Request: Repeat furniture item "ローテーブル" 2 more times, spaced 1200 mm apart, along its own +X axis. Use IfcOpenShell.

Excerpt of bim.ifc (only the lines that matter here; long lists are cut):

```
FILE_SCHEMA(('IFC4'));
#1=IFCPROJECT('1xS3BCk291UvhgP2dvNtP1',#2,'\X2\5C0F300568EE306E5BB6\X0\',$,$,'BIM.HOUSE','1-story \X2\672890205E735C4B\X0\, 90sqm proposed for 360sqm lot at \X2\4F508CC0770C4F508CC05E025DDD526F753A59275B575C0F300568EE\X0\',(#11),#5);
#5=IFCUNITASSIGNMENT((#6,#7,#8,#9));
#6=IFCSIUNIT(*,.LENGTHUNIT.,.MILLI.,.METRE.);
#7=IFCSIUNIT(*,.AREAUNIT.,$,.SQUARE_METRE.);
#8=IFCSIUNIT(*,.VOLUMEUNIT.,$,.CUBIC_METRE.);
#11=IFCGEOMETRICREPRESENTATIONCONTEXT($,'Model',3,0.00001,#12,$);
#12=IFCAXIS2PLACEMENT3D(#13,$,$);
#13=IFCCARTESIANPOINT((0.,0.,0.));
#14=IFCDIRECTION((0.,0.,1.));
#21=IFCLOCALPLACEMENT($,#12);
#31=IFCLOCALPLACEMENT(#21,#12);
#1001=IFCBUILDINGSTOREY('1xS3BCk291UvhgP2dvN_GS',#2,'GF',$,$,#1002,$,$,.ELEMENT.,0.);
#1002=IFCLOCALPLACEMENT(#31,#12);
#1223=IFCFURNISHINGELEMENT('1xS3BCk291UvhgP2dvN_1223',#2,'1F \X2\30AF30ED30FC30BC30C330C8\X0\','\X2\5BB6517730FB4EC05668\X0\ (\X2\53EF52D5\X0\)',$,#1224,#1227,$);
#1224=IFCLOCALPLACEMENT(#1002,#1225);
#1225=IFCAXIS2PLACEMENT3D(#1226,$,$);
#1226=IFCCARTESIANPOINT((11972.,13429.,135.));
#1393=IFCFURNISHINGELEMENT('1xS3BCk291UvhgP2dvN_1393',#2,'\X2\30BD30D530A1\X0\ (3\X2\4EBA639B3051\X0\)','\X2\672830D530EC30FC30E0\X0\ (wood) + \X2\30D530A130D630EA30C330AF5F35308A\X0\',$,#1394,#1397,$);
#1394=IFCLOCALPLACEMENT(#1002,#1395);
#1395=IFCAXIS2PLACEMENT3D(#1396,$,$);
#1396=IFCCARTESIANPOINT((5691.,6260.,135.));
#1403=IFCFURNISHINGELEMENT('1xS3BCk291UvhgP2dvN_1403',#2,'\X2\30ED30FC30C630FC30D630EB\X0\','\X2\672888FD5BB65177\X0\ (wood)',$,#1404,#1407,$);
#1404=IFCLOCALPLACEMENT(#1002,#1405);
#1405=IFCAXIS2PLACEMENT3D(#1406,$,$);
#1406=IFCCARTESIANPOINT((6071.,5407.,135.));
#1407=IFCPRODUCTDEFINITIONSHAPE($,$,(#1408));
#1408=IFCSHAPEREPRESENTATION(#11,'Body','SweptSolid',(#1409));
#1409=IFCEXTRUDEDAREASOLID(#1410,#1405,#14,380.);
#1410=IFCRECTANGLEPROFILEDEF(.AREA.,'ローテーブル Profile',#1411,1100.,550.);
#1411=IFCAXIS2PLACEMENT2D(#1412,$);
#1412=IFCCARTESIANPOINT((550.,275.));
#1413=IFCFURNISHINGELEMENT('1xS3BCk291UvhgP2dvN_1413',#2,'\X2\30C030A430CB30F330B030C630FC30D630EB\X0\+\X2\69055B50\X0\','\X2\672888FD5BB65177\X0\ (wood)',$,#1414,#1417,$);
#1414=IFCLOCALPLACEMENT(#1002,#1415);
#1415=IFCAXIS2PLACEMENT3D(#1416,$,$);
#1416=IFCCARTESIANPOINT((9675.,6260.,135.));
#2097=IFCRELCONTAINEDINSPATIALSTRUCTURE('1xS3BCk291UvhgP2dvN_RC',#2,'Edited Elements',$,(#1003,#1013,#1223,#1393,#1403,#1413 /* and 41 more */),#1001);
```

```python
import ifcopenshell
import ifcopenshell.api.geometry
import ifcopenshell.api.root
import ifcopenshell.util.element
import ifcopenshell.util.placement
import ifcopenshell.util.unit

model = ifcopenshell.open("bim.ifc")
unit_scale = ifcopenshell.util.unit.calculate_unit_scale(model)


def reuse_history(source, copy):
    """copy_class also copies each property set's owner history, people and application; keep the originals."""
    for rel in copy.IsDefinedBy:
        if rel.is_a("IfcRelDefinesByProperties") and (history := rel.RelatingPropertyDefinition.OwnerHistory):
            rel.RelatingPropertyDefinition.OwnerHistory = source.OwnerHistory
            ifcopenshell.util.element.remove_deep2(model, history)


source = model.by_id(1403)
base = ifcopenshell.util.placement.get_local_placement(source.ObjectPlacement)
step = base[:3, 0] * 1.2 / unit_scale

for i in range(1, 3):
    copy = ifcopenshell.api.root.copy_class(model, product=source)
    copy.Representation = ifcopenshell.util.element.copy_deep(
        model, source.Representation, exclude=["IfcGeometricRepresentationContext", "IfcRepresentationMap"]
    )
    reuse_history(source, copy)
    matrix = base.copy()
    matrix[:3, 3] += i * step
    print("added at", matrix[:3, 3].round(3) + 0.0)
    ifcopenshell.api.geometry.edit_object_placement(model, product=copy, matrix=matrix, is_si=False)

model.write("bim_v2.ifc")
```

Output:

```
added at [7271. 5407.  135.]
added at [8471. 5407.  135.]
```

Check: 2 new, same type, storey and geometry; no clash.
